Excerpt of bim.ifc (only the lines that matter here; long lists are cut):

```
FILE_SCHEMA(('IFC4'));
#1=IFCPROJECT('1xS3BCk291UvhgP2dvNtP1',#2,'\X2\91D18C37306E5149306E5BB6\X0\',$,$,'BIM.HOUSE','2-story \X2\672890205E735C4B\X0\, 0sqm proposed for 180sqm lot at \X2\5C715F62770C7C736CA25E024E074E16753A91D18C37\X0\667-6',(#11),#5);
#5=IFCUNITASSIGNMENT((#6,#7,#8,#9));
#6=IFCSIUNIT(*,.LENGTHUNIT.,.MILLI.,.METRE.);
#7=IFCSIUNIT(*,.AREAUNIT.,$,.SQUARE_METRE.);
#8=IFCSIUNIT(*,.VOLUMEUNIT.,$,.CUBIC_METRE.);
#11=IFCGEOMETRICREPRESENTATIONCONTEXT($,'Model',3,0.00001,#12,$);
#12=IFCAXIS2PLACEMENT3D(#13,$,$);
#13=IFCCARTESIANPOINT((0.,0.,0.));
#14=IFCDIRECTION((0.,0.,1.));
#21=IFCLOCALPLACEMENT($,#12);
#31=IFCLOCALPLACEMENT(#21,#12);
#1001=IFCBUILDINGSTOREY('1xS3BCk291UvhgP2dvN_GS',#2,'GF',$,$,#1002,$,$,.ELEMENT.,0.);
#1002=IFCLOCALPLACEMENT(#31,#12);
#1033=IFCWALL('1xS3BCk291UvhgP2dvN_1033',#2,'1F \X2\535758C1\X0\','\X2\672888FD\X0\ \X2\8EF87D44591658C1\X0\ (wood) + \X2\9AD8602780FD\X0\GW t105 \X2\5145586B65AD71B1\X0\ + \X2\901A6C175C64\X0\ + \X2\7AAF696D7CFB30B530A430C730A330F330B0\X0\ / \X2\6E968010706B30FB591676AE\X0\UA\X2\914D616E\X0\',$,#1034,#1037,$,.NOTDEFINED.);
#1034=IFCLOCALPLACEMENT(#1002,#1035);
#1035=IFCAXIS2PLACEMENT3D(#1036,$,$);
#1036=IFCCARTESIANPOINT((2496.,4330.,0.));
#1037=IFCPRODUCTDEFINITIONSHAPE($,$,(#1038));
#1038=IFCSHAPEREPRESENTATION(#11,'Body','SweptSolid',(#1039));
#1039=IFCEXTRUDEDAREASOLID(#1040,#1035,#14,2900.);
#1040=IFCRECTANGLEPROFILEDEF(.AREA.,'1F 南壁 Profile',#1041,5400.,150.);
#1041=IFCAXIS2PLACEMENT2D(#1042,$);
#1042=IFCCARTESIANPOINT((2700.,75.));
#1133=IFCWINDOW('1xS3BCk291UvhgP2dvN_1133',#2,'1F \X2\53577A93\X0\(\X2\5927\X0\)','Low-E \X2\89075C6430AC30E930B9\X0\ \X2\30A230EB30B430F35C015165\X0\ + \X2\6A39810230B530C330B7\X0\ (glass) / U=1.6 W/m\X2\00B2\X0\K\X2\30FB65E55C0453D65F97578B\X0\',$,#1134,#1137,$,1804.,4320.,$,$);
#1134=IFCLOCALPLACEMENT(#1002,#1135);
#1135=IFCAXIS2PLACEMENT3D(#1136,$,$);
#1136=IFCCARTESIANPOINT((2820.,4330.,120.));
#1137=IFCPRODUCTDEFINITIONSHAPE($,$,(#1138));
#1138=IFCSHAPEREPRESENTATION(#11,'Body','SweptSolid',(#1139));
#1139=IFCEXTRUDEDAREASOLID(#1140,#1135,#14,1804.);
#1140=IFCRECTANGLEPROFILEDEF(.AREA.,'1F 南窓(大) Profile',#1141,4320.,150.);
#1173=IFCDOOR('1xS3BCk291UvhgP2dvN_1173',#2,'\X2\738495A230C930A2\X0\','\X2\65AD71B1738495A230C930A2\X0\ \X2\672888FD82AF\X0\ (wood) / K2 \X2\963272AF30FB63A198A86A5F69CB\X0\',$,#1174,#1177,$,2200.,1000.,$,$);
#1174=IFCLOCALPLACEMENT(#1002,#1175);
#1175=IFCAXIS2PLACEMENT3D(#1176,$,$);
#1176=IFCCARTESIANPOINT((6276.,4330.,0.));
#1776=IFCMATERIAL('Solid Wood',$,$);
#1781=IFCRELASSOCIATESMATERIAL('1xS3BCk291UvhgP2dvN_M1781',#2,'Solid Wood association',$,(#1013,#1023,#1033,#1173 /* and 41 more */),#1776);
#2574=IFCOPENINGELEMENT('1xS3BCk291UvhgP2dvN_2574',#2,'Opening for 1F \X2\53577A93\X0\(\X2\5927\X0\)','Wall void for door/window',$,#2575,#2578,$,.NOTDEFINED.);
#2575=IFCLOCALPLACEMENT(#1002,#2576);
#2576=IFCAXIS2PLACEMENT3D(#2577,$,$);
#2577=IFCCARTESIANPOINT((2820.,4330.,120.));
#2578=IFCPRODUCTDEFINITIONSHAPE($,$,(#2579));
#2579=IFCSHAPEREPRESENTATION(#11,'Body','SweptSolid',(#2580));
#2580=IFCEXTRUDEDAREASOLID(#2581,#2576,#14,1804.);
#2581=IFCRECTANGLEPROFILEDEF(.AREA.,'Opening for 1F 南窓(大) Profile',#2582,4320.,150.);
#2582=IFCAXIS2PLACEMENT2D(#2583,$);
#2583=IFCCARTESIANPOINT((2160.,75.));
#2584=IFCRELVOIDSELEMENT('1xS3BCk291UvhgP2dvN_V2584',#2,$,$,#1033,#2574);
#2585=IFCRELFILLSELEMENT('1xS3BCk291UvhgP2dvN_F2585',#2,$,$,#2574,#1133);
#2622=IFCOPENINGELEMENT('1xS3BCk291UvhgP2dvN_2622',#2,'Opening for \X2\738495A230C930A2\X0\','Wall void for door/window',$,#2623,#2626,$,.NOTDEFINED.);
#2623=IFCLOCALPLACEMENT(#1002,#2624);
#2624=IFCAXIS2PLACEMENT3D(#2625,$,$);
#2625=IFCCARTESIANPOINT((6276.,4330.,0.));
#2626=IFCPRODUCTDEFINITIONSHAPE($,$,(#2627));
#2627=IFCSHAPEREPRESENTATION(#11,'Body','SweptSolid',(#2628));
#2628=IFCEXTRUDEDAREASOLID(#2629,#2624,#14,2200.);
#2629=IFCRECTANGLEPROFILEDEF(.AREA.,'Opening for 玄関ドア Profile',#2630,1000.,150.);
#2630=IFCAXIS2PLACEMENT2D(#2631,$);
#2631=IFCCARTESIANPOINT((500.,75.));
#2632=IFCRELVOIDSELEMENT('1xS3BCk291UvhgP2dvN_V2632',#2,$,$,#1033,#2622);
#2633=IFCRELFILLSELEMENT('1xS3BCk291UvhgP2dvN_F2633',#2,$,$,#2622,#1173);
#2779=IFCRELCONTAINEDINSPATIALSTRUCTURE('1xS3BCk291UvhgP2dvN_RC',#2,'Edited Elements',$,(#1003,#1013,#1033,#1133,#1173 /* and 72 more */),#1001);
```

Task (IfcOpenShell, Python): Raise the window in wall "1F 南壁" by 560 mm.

```python
import numpy as np
import ifcopenshell
import ifcopenshell.api.geometry
import ifcopenshell.util.placement
import ifcopenshell.util.unit

model = ifcopenshell.open("bim.ifc")
unit_scale = ifcopenshell.util.unit.calculate_unit_scale(model)

window = model.by_id(1133)
opening = window.FillsVoids[0].RelatingOpeningElement
dz = 0.56 / unit_scale

shift = np.array([0.0, 0.0, dz])
# The window is not placed relative to its opening, so move both.
for product in (opening, window):
    matrix = ifcopenshell.util.placement.get_local_placement(product.ObjectPlacement)
    matrix[:3, 3] += shift
    ifcopenshell.api.geometry.edit_object_placement(model, product=product, matrix=matrix, is_si=False)

print(f"moved by {dz * unit_scale:+.3f} m")

model.write("bim_v2.ifc")
```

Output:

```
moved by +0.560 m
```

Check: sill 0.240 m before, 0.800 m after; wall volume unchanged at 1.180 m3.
